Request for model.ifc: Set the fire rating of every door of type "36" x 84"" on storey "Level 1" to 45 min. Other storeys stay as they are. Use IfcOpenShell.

First a look at what the model holds.

```python
import ifcopenshell
import ifcopenshell.util.element

model = ifcopenshell.open("model.ifc")
print(model.schema)
storey = next(s for s in model.by_type("IfcBuildingStorey") if s.Name == "Level 1")
doors = [e for e in ifcopenshell.util.element.get_decomposition(storey) if e.is_a("IfcDoor")]
seen = {}
for e in doors:
    element_type = ifcopenshell.util.element.get_type(e)
    key = (element_type.Name if element_type != e and element_type else None, ifcopenshell.util.element.get_pset(e, "Pset_DoorCommon", "FireRating"))
    seen[key] = seen.get(key, 0) + 1
for (name, value), count in sorted(seen.items(), key=str):
    print(count, "x", name, "|", value)
```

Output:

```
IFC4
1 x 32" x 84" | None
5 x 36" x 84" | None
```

```python
import ifcopenshell
import ifcopenshell.api.pset
import ifcopenshell.util.element

model = ifcopenshell.open("model.ifc")

storey = next(s for s in model.by_type("IfcBuildingStorey") if s.Name == "Level 1")
doors = [e for e in ifcopenshell.util.element.get_decomposition(storey) if e.is_a("IfcDoor")]

count = 0
for e in doors:
    element_type = ifcopenshell.util.element.get_type(e)
    if element_type in (None, e) or element_type.Name != '36" x 84"':
        continue
    # add_pset returns the element's existing set when there is one.
    pset = ifcopenshell.api.pset.add_pset(model, product=e, name="Pset_DoorCommon")
    ifcopenshell.api.pset.edit_pset(model, pset=pset, properties={"FireRating": "45 min"})
    count += 1

print(count, "doors updated")

model.write("model-out.ifc")
```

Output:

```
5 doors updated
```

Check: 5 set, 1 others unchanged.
